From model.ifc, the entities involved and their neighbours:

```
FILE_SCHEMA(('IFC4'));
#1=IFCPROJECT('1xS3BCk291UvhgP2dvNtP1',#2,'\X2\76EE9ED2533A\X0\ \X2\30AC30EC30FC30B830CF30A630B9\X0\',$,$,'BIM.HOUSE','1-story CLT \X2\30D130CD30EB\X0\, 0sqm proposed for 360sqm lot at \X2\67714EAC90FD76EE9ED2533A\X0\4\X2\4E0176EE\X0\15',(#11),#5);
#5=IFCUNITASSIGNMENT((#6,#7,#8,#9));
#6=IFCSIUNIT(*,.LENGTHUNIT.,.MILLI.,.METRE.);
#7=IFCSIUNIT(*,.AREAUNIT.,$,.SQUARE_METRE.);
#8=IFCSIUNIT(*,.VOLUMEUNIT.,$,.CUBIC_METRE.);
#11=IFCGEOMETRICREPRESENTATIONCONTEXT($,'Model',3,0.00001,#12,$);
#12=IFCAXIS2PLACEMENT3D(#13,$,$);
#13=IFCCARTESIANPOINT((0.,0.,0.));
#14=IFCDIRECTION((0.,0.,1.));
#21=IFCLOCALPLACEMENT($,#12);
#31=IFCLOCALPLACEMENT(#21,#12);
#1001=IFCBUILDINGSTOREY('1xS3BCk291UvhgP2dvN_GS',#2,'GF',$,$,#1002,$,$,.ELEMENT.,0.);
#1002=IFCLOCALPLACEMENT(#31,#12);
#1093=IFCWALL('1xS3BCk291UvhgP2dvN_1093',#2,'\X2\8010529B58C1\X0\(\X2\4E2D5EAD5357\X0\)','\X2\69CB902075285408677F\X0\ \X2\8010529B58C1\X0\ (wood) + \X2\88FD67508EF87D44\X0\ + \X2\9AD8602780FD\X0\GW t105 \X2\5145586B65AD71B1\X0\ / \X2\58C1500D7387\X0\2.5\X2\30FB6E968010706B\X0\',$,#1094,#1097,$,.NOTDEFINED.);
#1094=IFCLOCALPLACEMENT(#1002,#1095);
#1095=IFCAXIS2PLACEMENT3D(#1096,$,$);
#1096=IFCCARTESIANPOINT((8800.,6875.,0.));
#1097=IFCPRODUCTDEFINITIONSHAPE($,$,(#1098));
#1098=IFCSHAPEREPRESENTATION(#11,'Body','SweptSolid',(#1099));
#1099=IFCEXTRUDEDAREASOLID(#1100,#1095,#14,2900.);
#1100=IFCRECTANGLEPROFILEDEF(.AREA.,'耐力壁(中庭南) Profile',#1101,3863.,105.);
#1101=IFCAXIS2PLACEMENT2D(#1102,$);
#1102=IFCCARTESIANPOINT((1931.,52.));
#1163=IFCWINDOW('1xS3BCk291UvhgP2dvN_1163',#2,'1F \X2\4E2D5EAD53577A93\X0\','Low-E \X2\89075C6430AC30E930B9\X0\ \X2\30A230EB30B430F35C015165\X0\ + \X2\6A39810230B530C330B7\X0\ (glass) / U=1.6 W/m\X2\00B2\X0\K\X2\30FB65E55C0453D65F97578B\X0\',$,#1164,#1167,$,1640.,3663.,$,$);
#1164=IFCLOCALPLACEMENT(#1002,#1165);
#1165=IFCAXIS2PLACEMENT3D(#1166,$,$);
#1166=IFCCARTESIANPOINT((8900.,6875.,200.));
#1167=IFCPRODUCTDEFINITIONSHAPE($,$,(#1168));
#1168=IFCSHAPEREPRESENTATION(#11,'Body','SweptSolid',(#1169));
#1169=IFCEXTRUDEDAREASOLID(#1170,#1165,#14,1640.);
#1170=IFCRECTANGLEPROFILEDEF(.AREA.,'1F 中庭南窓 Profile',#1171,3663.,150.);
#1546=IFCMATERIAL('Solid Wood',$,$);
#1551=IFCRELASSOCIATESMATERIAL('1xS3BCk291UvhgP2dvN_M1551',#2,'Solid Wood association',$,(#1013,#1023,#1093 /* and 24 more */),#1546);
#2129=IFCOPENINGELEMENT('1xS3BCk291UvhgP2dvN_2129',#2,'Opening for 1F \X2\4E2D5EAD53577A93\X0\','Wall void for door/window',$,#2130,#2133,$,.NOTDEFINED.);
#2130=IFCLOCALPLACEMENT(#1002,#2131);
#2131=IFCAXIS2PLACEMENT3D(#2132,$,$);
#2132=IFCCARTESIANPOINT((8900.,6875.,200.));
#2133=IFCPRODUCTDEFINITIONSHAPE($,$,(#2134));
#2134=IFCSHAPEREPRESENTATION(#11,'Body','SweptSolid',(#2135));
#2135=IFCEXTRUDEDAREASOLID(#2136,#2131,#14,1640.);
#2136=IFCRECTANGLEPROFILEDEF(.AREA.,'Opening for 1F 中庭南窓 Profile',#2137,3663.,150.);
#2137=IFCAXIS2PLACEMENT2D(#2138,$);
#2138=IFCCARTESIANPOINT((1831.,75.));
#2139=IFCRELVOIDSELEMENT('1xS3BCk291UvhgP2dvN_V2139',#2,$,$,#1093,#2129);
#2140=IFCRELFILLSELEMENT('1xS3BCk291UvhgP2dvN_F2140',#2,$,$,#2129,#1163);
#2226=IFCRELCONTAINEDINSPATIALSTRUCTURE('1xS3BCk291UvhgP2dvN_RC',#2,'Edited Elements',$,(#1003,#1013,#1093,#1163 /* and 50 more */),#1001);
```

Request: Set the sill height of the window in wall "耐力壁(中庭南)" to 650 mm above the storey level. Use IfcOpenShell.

```python
import numpy as np
import ifcopenshell
import ifcopenshell.api.geometry
import ifcopenshell.geom
import ifcopenshell.util.element
import ifcopenshell.util.placement
import ifcopenshell.util.shape
import ifcopenshell.util.unit

model = ifcopenshell.open("model.ifc")
unit_scale = ifcopenshell.util.unit.calculate_unit_scale(model)

window = model.by_id(1163)
opening = window.FillsVoids[0].RelatingOpeningElement
storey = ifcopenshell.util.element.get_container(window, ifc_class="IfcBuildingStorey")
level = ifcopenshell.util.placement.get_local_placement(storey.ObjectPlacement)[2, 3]

# The opening's origin need not be at the sill, so measure its lowest point.
shape = ifcopenshell.geom.create_shape(ifcopenshell.geom.settings(), opening)
bottom = ifcopenshell.util.shape.get_shape_bottom_elevation(shape, shape.geometry) / unit_scale
dz = level + 650.0 - bottom

shift = np.array([0.0, 0.0, dz])
# The window is not placed relative to its opening, so move both.
for product in (opening, window):
    matrix = ifcopenshell.util.placement.get_local_placement(product.ObjectPlacement)
    matrix[:3, 3] += shift
    ifcopenshell.api.geometry.edit_object_placement(model, product=product, matrix=matrix, is_si=False)

print(f"moved by {dz * unit_scale:+.3f} m")

model.write("model_v2.ifc")
```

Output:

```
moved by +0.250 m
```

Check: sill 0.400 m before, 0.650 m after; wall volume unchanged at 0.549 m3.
